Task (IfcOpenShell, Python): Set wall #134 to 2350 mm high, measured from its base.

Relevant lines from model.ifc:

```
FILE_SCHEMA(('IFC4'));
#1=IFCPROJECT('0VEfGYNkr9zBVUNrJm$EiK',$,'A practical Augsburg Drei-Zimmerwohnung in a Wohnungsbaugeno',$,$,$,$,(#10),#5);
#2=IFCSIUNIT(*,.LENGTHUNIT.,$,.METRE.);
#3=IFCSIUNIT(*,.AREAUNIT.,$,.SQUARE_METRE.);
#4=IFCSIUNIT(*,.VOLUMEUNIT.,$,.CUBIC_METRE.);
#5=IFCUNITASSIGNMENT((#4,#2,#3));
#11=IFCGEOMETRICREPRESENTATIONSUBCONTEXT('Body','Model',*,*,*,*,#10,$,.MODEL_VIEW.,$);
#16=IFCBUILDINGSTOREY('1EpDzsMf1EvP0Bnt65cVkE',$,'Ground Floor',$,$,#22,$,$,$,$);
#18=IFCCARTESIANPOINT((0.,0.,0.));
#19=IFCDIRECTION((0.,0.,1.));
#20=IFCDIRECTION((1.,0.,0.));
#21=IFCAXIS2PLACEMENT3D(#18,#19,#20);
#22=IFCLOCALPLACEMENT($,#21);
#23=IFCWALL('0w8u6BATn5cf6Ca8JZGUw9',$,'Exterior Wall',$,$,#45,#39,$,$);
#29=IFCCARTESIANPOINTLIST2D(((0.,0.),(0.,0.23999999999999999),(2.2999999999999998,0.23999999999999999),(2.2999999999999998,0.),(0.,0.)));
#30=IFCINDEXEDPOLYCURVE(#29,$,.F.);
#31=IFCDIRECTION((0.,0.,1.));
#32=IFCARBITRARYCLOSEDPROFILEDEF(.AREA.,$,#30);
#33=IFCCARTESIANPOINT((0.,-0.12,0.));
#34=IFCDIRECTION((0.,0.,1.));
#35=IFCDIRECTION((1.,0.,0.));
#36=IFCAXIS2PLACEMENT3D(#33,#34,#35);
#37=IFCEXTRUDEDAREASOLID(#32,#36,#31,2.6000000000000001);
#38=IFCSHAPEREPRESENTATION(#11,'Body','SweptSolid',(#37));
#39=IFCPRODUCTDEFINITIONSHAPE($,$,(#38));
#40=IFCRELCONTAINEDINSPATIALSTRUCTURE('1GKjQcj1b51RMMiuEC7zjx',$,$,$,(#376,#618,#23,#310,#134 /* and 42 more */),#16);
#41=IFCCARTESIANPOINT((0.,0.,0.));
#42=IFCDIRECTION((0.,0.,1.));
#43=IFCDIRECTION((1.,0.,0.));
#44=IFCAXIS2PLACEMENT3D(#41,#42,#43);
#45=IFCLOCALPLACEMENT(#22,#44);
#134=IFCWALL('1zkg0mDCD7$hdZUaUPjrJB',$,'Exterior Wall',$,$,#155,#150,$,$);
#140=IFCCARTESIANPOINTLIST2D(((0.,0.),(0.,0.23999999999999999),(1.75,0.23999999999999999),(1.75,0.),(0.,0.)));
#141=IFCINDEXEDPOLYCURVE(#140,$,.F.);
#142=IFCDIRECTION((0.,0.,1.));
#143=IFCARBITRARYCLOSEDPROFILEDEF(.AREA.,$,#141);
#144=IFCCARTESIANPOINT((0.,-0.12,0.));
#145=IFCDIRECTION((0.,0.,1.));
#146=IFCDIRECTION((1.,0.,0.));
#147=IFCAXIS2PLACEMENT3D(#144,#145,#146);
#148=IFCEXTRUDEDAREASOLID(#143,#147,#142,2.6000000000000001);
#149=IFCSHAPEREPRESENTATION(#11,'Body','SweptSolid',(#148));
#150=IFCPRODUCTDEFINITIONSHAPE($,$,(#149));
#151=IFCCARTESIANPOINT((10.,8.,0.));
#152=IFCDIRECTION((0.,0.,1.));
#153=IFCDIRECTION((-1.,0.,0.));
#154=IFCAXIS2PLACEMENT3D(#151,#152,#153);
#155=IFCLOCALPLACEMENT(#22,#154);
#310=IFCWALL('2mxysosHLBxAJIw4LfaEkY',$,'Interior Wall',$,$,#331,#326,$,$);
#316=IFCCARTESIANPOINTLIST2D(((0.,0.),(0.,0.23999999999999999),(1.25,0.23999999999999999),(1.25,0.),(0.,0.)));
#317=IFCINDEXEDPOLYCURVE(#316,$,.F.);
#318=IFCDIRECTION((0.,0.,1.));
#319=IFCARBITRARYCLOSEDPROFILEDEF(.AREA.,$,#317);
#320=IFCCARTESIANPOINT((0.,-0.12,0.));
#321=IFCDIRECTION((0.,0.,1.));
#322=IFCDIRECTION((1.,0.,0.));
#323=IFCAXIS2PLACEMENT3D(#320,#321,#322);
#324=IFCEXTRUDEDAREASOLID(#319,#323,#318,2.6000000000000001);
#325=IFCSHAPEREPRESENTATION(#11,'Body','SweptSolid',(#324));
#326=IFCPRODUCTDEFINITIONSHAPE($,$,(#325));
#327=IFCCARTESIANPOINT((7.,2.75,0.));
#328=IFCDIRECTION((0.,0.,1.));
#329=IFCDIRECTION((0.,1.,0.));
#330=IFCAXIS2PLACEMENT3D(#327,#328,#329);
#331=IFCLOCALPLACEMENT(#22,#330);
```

```python
import ifcopenshell
import ifcopenshell.geom
import ifcopenshell.util.representation
import ifcopenshell.util.shape
import ifcopenshell.util.unit

model = ifcopenshell.open("model.ifc")
unit_scale = ifcopenshell.util.unit.calculate_unit_scale(model)
settings = ifcopenshell.geom.settings()


def volume(element):
    """Net volume in cubic metres, openings subtracted."""
    shape = ifcopenshell.geom.create_shape(settings, element)
    return ifcopenshell.util.shape.get_volume(shape.geometry)


wall = model.by_guid("1zkg0mDCD7$hdZUaUPjrJB")
before = volume(wall)

body = ifcopenshell.util.representation.get_representation(wall, "Model", "Body")
solid = body.Items[0]
old_height = solid.Depth
solid.Depth = 2.35 / unit_scale
after = volume(wall)

print(f"height {old_height:g} -> {solid.Depth:g}, volume {before:.3f} -> {after:.3f} m3")

model.write("model_updated.ifc")
```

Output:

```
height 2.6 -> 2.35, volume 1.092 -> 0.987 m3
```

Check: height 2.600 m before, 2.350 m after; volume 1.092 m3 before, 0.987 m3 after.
